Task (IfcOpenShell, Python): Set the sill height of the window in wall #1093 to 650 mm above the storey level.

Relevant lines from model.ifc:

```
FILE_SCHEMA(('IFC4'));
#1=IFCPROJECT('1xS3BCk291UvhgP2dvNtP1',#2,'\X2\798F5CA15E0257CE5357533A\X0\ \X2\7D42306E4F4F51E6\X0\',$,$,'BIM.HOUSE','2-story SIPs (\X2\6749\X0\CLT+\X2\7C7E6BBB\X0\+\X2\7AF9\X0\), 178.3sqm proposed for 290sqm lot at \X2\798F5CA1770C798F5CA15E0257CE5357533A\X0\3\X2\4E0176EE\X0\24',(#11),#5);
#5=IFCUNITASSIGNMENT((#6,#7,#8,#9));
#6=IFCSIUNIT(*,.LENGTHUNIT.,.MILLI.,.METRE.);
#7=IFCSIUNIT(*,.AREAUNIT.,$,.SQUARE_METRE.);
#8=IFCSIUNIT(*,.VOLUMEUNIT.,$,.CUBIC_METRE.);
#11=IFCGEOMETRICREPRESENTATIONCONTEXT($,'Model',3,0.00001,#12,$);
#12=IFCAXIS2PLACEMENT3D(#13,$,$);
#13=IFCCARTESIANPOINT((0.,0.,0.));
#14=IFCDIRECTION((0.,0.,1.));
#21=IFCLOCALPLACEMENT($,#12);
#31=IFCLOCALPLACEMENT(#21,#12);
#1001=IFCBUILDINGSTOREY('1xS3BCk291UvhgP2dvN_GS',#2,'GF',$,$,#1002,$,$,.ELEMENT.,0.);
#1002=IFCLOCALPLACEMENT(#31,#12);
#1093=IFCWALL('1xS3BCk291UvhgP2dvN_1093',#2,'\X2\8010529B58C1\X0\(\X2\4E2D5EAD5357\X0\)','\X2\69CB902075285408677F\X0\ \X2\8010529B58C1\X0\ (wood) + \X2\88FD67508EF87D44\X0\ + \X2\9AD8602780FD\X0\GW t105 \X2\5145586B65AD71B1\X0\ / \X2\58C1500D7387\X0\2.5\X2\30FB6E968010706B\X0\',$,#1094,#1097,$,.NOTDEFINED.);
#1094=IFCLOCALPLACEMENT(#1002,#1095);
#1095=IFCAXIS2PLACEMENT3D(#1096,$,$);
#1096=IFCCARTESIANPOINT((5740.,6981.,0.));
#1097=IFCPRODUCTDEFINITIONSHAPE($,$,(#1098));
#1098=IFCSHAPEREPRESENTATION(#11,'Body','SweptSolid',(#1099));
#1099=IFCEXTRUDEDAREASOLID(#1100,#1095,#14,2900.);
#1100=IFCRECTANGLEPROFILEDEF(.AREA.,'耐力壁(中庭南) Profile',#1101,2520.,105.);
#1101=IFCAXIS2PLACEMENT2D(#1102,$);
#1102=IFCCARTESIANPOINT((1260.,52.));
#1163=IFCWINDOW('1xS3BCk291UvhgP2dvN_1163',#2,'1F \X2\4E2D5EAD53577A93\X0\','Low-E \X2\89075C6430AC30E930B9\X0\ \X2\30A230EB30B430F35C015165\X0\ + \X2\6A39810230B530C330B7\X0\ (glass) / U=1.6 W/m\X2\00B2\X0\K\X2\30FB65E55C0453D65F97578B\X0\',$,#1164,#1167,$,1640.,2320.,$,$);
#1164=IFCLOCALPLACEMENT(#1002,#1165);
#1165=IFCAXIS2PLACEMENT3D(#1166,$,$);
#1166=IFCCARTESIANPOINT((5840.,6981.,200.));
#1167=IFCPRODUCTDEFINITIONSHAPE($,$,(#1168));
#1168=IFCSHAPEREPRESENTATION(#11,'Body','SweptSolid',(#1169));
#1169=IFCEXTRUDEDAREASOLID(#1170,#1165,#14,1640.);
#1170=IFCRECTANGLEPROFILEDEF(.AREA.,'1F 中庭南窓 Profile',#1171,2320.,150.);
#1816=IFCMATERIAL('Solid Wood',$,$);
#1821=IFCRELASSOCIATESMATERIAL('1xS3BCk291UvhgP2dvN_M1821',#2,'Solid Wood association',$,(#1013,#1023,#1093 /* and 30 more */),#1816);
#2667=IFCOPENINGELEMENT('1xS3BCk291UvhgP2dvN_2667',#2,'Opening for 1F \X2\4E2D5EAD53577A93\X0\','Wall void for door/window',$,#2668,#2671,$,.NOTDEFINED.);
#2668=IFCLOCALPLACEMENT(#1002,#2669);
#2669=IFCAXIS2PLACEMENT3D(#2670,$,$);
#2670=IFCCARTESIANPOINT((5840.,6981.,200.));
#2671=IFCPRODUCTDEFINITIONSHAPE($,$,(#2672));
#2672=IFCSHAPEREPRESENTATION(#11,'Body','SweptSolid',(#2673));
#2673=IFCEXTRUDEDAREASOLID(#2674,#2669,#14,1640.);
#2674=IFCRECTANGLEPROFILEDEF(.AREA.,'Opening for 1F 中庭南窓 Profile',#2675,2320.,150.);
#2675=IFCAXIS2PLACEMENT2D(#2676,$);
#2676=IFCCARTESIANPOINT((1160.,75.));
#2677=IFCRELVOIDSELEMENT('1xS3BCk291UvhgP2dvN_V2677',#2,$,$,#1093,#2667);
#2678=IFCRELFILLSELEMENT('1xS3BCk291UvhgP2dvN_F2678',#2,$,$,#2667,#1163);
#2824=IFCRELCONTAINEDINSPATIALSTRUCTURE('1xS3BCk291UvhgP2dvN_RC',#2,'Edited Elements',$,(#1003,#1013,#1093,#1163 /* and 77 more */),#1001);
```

```python
import numpy as np
import ifcopenshell
import ifcopenshell.api.geometry
import ifcopenshell.geom
import ifcopenshell.util.element
import ifcopenshell.util.placement
import ifcopenshell.util.shape
import ifcopenshell.util.unit

model = ifcopenshell.open("model.ifc")
unit_scale = ifcopenshell.util.unit.calculate_unit_scale(model)

window = model.by_guid("1xS3BCk291UvhgP2dvN_1163")
opening = window.FillsVoids[0].RelatingOpeningElement
storey = ifcopenshell.util.element.get_container(window, ifc_class="IfcBuildingStorey")
level = ifcopenshell.util.placement.get_local_placement(storey.ObjectPlacement)[2, 3]

# The opening's origin need not be at the sill, so measure its lowest point.
shape = ifcopenshell.geom.create_shape(ifcopenshell.geom.settings(), opening)
bottom = ifcopenshell.util.shape.get_shape_bottom_elevation(shape, shape.geometry) / unit_scale
dz = level + 0.65 / unit_scale - bottom

shift = np.array([0.0, 0.0, dz])
# The window is not placed relative to its opening, so move both.
for product in (opening, window):
    matrix = ifcopenshell.util.placement.get_local_placement(product.ObjectPlacement)
    matrix[:3, 3] += shift
    ifcopenshell.api.geometry.edit_object_placement(model, product=product, matrix=matrix, is_si=False)

print(f"moved by {dz * unit_scale:+.3f} m")

model.write("model-out.ifc")
```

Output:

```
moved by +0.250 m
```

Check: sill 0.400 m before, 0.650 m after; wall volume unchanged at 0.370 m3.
